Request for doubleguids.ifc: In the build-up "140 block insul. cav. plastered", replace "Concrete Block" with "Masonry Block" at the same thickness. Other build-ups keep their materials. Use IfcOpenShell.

First a look at what the model holds.

```python
import ifcopenshell
import ifcopenshell.util.element

model = ifcopenshell.open("doubleguids.ifc")
print(model.schema)
for layer_set in model.by_type("IfcMaterialLayerSet"):
    if layer_set.LayerSetName == "140 block insul. cav. plastered":
        for layer in layer_set.MaterialLayers:
            print(layer.id(), layer.Material and layer.Material.Name, layer.LayerThickness, sep=" | ")
        print(len(ifcopenshell.util.element.get_elements_by_material(model, layer_set)), "elements and types use it")
print(sorted(m.Name for m in model.by_type("IfcMaterial") if m.Name)[:60])
```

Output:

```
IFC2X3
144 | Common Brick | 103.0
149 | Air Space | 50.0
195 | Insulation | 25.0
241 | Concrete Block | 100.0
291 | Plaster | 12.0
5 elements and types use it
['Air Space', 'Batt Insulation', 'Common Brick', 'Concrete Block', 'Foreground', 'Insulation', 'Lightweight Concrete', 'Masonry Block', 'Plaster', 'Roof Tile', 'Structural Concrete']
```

```python
import ifcopenshell
import ifcopenshell.api.material

model = ifcopenshell.open("doubleguids.ifc")

layer_set = next(s for s in model.by_type("IfcMaterialLayerSet") if s.LayerSetName == "140 block insul. cav. plastered")
layer = next(l for l in layer_set.MaterialLayers if l.Material and l.Material.Name == "Concrete Block")
material = next(m for m in model.by_type("IfcMaterial") if m.Name == "Masonry Block")

# Point this one layer at the other material; renaming the old one would change it everywhere.
ifcopenshell.api.material.edit_layer(model, layer=layer, attributes={}, material=material)

print([l.Material.Name if l.Material else None for l in layer_set.MaterialLayers])

model.write("doubleguids-out.ifc")
```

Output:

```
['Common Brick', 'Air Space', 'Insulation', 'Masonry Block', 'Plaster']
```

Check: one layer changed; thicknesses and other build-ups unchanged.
